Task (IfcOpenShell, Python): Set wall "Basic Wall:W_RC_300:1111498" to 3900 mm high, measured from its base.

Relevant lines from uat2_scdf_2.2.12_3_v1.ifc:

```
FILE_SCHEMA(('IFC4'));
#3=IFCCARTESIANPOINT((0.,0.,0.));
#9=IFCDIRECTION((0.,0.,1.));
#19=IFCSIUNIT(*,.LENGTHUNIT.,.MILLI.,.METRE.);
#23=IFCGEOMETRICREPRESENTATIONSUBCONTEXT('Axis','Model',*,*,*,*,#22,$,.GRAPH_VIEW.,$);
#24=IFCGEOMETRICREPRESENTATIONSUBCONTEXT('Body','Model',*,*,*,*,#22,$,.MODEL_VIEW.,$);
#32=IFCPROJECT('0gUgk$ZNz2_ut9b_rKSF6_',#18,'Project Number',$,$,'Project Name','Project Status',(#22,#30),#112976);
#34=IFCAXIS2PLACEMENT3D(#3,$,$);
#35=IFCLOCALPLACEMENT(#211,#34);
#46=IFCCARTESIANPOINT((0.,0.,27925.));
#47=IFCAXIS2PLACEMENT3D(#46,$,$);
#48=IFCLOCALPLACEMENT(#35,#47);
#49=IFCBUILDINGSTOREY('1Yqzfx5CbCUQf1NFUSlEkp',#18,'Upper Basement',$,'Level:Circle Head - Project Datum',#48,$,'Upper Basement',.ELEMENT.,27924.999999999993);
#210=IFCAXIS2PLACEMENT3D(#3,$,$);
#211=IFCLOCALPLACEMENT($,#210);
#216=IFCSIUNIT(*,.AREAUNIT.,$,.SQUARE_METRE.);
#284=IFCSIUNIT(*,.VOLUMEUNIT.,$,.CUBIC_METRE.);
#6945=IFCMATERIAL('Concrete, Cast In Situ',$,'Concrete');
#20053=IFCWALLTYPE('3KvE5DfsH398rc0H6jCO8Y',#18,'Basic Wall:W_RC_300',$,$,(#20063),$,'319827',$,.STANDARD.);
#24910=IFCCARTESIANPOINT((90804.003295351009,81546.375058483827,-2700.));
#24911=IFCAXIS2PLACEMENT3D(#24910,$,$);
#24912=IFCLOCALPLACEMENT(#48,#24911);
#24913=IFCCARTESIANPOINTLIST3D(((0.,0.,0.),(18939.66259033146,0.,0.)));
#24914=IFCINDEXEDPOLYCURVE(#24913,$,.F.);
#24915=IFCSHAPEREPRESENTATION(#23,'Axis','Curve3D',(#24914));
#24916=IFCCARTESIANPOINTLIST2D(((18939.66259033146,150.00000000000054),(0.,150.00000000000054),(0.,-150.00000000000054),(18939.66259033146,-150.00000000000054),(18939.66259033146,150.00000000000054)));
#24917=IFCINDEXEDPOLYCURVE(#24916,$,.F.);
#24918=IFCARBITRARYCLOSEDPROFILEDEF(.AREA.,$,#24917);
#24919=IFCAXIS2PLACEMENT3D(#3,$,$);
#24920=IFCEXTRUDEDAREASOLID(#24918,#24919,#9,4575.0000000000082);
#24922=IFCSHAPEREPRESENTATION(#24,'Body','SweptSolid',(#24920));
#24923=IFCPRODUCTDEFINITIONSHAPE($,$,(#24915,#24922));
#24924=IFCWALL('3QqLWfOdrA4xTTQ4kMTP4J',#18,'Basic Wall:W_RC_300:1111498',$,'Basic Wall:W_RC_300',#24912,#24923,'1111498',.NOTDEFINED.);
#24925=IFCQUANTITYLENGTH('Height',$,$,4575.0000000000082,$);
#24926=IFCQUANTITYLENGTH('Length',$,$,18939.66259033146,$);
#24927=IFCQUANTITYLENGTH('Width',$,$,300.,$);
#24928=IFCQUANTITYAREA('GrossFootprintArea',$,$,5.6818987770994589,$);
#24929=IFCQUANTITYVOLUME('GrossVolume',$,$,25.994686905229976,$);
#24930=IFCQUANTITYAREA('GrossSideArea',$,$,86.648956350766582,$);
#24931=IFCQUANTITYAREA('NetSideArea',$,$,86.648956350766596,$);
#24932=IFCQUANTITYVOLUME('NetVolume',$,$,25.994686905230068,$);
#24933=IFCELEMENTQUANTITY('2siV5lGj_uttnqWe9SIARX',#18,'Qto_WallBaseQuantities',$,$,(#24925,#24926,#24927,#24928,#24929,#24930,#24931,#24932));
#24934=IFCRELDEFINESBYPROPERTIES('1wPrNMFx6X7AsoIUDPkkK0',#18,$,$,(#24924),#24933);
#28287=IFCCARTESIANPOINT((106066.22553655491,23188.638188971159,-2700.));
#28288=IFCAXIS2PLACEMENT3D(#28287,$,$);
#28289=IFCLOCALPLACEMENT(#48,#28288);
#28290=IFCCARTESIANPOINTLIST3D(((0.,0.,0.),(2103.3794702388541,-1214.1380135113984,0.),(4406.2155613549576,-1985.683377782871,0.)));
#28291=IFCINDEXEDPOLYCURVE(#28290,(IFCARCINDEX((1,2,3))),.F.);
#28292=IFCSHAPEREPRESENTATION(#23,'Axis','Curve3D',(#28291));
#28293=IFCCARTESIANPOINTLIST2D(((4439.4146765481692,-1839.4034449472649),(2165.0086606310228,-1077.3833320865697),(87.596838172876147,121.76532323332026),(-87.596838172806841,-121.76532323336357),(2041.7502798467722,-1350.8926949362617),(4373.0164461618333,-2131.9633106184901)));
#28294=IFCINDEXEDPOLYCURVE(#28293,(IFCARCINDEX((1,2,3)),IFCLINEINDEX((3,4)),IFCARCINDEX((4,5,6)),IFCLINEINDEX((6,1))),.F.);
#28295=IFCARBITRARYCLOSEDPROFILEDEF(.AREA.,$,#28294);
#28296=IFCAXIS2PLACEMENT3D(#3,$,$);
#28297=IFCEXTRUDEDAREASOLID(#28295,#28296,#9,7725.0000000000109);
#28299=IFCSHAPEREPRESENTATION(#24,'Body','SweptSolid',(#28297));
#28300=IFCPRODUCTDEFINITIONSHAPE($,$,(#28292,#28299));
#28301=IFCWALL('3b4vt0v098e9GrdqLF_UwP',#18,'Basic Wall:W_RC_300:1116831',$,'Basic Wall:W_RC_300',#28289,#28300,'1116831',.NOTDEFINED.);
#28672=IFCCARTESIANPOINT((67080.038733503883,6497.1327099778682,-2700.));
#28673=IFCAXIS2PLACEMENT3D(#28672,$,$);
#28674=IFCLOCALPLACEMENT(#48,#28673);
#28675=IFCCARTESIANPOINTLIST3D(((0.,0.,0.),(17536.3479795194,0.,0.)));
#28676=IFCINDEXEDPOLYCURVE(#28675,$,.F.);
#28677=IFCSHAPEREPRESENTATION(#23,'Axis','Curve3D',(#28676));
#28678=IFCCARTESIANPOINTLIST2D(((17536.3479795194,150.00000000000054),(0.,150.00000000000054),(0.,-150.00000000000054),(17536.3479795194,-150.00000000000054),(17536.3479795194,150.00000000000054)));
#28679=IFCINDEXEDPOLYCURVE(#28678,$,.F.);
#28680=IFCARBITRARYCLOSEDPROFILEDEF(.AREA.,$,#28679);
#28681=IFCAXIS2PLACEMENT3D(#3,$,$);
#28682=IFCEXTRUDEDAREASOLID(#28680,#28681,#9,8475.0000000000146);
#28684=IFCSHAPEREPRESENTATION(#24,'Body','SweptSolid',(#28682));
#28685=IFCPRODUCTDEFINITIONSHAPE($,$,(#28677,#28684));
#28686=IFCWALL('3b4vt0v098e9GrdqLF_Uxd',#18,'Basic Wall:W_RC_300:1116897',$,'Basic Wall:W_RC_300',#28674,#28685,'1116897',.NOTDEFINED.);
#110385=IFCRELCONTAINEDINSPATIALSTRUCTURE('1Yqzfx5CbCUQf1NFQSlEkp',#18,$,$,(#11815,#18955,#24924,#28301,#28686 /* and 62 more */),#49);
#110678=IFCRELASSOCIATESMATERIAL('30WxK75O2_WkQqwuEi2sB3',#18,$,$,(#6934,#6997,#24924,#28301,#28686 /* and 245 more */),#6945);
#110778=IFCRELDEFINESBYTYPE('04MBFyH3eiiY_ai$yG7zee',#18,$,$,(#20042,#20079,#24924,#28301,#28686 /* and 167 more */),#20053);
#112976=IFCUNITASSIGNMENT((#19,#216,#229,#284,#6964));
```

```python
import ifcopenshell
import ifcopenshell.api.pset
import ifcopenshell.geom
import ifcopenshell.util.element
import ifcopenshell.util.representation
import ifcopenshell.util.shape
import ifcopenshell.util.unit

model = ifcopenshell.open("uat2_scdf_2.2.12_3_v1.ifc")
unit_scale = ifcopenshell.util.unit.calculate_unit_scale(model)
area_scale = ifcopenshell.util.unit.calculate_unit_scale(model, "AREAUNIT")
volume_scale = ifcopenshell.util.unit.calculate_unit_scale(model, "VOLUMEUNIT")
settings = ifcopenshell.geom.settings()


def volume(element):
    """Net volume in cubic metres, openings subtracted."""
    shape = ifcopenshell.geom.create_shape(settings, element)
    return ifcopenshell.util.shape.get_volume(shape.geometry)


wall = model.by_id(24924)
before = volume(wall)

body = ifcopenshell.util.representation.get_representation(wall, "Model", "Body")
solid = body.Items[0]
old_height = solid.Depth
solid.Depth = 3900.0
after = volume(wall)
thickness = 0.3  # wall thickness in metres

# Update the stored height, areas and volumes.
qto = model.by_id(ifcopenshell.util.element.get_pset(wall, "Qto_WallBaseQuantities", should_inherit=False)["id"])
ifcopenshell.api.pset.edit_qto(model, qto=qto, properties={
    "Height": solid.Depth,
    "GrossVolume": ifcopenshell.util.element.get_pset(wall, "Qto_WallBaseQuantities", "GrossVolume") * solid.Depth / old_height,
    "GrossSideArea": ifcopenshell.util.element.get_pset(wall, "Qto_WallBaseQuantities", "GrossSideArea") * solid.Depth / old_height,
    "NetSideArea": after / thickness / area_scale,
    "NetVolume": after / volume_scale,
})

print(f"height {old_height:g} -> {solid.Depth:g}, volume {before:.3f} -> {after:.3f} m3")

model.write("uat2_scdf_2.2.12_3_v1-out.ifc")
```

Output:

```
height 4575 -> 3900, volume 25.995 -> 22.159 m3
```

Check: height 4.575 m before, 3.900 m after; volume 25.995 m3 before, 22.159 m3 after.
